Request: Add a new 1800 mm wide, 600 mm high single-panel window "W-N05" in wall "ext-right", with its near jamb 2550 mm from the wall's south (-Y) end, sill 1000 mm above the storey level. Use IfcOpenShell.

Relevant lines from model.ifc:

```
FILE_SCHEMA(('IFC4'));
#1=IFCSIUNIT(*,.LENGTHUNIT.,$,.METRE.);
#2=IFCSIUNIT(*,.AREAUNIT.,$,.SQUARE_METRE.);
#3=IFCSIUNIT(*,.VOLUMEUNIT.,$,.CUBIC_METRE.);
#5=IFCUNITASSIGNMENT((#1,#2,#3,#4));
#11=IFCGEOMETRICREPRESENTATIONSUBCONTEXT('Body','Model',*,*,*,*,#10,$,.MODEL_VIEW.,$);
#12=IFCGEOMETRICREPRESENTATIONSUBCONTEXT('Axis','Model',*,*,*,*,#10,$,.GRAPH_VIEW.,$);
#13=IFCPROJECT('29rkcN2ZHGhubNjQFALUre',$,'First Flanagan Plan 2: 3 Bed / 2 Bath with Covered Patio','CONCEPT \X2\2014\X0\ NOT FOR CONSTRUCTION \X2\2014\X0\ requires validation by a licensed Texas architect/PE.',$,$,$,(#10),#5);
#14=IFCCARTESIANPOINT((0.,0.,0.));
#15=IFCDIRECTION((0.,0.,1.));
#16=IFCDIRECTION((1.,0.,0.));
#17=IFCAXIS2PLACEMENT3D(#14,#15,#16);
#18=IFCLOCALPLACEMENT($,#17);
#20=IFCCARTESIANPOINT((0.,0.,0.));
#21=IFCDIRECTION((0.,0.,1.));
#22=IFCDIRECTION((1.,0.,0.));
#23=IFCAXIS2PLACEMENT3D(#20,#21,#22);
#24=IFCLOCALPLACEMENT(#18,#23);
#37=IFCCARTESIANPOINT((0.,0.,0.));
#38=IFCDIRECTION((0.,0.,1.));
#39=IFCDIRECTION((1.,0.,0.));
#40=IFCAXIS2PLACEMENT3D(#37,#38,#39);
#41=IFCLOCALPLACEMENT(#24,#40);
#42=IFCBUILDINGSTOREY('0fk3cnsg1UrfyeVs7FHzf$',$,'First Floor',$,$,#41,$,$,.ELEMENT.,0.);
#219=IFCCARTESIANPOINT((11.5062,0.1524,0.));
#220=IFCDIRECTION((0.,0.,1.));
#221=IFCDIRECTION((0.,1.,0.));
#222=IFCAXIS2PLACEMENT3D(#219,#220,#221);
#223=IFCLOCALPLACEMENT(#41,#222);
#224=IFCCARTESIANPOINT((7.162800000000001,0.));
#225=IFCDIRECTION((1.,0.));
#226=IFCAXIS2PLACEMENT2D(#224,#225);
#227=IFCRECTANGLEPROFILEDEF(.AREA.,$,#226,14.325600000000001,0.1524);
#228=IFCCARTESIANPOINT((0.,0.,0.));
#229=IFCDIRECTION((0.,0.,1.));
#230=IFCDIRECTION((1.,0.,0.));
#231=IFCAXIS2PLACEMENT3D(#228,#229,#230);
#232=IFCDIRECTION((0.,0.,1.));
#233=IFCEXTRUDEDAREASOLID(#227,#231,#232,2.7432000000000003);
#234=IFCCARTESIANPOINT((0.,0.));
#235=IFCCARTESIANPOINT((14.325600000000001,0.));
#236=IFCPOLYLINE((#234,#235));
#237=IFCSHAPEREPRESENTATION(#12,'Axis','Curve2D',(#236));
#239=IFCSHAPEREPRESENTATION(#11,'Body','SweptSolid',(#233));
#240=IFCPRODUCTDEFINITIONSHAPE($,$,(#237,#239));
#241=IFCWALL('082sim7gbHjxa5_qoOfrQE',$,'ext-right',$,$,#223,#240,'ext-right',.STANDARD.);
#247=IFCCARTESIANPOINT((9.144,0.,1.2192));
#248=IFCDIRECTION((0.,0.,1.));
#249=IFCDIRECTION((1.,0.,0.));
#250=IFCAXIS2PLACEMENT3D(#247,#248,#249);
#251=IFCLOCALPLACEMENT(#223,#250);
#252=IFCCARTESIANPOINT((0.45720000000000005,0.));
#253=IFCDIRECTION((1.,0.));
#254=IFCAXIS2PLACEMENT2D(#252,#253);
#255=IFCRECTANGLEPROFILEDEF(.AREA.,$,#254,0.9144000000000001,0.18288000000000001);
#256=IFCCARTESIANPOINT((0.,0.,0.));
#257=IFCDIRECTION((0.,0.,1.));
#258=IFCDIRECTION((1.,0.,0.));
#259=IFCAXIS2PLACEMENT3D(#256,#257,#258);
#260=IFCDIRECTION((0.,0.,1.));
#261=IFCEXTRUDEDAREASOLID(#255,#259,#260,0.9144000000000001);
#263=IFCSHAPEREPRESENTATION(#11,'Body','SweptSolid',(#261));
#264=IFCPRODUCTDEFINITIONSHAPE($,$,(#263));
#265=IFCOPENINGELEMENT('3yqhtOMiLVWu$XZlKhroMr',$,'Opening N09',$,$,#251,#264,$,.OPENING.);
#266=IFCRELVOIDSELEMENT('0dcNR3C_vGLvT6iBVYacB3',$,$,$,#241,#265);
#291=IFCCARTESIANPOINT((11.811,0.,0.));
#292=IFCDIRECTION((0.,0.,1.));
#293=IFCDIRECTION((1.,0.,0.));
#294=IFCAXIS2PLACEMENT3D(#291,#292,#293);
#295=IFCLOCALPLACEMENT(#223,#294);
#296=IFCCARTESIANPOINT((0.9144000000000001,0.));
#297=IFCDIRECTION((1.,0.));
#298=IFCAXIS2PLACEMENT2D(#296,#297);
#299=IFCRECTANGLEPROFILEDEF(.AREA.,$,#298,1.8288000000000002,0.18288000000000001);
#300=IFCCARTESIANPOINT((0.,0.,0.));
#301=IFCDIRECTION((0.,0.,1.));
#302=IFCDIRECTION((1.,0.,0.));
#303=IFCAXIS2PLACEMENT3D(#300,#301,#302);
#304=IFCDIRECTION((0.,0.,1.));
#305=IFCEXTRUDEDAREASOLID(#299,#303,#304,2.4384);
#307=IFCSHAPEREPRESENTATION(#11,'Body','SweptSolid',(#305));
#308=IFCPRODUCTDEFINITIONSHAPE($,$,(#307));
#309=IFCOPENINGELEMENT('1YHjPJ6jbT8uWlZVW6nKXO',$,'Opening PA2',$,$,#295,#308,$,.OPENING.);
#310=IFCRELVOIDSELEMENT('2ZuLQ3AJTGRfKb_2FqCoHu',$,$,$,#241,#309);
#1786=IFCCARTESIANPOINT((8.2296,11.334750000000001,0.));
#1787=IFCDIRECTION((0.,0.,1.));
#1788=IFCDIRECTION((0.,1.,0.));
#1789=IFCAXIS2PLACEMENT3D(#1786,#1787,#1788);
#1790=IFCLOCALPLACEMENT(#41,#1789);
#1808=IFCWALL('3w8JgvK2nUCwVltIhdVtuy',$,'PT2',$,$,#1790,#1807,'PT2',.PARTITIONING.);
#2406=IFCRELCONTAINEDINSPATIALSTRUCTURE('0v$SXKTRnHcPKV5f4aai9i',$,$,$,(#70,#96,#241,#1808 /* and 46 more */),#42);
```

```python
import numpy as np
import ifcopenshell
import ifcopenshell.api.feature
import ifcopenshell.api.geometry
import ifcopenshell.api.root
import ifcopenshell.api.spatial
import ifcopenshell.geom
import ifcopenshell.util.element
import ifcopenshell.util.placement
import ifcopenshell.util.representation
import ifcopenshell.util.shape
import ifcopenshell.util.unit

model = ifcopenshell.open("model.ifc")
unit_scale = ifcopenshell.util.unit.calculate_unit_scale(model)
settings = ifcopenshell.geom.settings()


def volume(element):
    """Net volume in cubic metres, openings subtracted."""
    shape = ifcopenshell.geom.create_shape(settings, element)
    return ifcopenshell.util.shape.get_volume(shape.geometry)


wall = model.by_guid("082sim7gbHjxa5_qoOfrQE")
storey = ifcopenshell.util.element.get_container(wall, ifc_class="IfcBuildingStorey")
context = ifcopenshell.util.representation.get_context(model, "Model", "Body", "MODEL_VIEW")
before = volume(wall)

width, height, from_end, sill = 1.8, 0.6, 2.55, 1  # metres

# The wall runs along its own X axis, and the end named is its -X end.
wall_shape = ifcopenshell.geom.create_shape(settings, wall)
x, y, z = ifcopenshell.util.shape.get_vertices(wall_shape.geometry).T
start = x.min() + from_end
face, thickness = float(y.min()), float(y.max() - y.min())
wall_matrix = ifcopenshell.util.placement.get_local_placement(wall.ObjectPlacement)
level = ifcopenshell.util.placement.get_local_placement(storey.ObjectPlacement)[2, 3]


def in_wall(x, y):
    """Placement at x, y metres in the wall's axes, at sill height."""
    matrix = wall_matrix.copy()
    matrix[:, 3] = wall_matrix @ np.array([x / unit_scale, y / unit_scale, 0.0, 1.0])
    matrix[2, 3] = level + sill / unit_scale
    return matrix


# Opening: a box that overshoots both wall faces by 50 mm.
opening = ifcopenshell.api.root.create_entity(model, ifc_class="IfcOpeningElement", predefined_type="OPENING")
box = ifcopenshell.api.geometry.add_wall_representation(
    model, context=context, length=width, height=height, thickness=thickness + 0.1
)
ifcopenshell.api.geometry.assign_representation(model, product=opening, representation=box)
ifcopenshell.api.geometry.edit_object_placement(model, product=opening, matrix=in_wall(start, face - 0.05), is_si=False)
ifcopenshell.api.feature.add_feature(model, feature=opening, element=wall)

window = ifcopenshell.api.root.create_entity(model, ifc_class="IfcWindow", name="W-N05", predefined_type="WINDOW")
window.OverallWidth, window.OverallHeight = width / unit_scale, height / unit_scale
window.PartitioningType = "SINGLE_PANEL"
body = ifcopenshell.api.geometry.add_window_representation(
    model,
    context=context,
    overall_width=window.OverallWidth,
    overall_height=window.OverallHeight,
    partition_type="SINGLE_PANEL",
)
ifcopenshell.api.geometry.assign_representation(model, product=window, representation=body)
ifcopenshell.api.spatial.assign_container(model, products=[window], relating_structure=storey)
ifcopenshell.api.feature.add_filling(model, opening=opening, element=window)

# Centre the window in the wall's thickness.
ifcopenshell.api.geometry.edit_object_placement(model, product=window, matrix=in_wall(start, face), is_si=False)
window_shape = ifcopenshell.geom.create_shape(settings, window)
depth = ifcopenshell.util.shape.get_vertices(window_shape.geometry)[:, 1]
offset = face + thickness / 2 - (depth.min() + depth.max()) / 2
ifcopenshell.api.geometry.edit_object_placement(model, product=window, matrix=in_wall(start, offset), is_si=False)

after = volume(wall)

print(f"wall volume {before:.3f} -> {after:.3f} m3")

model.write("model_updated.ifc")
```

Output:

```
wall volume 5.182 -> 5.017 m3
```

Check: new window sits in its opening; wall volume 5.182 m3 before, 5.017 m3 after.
